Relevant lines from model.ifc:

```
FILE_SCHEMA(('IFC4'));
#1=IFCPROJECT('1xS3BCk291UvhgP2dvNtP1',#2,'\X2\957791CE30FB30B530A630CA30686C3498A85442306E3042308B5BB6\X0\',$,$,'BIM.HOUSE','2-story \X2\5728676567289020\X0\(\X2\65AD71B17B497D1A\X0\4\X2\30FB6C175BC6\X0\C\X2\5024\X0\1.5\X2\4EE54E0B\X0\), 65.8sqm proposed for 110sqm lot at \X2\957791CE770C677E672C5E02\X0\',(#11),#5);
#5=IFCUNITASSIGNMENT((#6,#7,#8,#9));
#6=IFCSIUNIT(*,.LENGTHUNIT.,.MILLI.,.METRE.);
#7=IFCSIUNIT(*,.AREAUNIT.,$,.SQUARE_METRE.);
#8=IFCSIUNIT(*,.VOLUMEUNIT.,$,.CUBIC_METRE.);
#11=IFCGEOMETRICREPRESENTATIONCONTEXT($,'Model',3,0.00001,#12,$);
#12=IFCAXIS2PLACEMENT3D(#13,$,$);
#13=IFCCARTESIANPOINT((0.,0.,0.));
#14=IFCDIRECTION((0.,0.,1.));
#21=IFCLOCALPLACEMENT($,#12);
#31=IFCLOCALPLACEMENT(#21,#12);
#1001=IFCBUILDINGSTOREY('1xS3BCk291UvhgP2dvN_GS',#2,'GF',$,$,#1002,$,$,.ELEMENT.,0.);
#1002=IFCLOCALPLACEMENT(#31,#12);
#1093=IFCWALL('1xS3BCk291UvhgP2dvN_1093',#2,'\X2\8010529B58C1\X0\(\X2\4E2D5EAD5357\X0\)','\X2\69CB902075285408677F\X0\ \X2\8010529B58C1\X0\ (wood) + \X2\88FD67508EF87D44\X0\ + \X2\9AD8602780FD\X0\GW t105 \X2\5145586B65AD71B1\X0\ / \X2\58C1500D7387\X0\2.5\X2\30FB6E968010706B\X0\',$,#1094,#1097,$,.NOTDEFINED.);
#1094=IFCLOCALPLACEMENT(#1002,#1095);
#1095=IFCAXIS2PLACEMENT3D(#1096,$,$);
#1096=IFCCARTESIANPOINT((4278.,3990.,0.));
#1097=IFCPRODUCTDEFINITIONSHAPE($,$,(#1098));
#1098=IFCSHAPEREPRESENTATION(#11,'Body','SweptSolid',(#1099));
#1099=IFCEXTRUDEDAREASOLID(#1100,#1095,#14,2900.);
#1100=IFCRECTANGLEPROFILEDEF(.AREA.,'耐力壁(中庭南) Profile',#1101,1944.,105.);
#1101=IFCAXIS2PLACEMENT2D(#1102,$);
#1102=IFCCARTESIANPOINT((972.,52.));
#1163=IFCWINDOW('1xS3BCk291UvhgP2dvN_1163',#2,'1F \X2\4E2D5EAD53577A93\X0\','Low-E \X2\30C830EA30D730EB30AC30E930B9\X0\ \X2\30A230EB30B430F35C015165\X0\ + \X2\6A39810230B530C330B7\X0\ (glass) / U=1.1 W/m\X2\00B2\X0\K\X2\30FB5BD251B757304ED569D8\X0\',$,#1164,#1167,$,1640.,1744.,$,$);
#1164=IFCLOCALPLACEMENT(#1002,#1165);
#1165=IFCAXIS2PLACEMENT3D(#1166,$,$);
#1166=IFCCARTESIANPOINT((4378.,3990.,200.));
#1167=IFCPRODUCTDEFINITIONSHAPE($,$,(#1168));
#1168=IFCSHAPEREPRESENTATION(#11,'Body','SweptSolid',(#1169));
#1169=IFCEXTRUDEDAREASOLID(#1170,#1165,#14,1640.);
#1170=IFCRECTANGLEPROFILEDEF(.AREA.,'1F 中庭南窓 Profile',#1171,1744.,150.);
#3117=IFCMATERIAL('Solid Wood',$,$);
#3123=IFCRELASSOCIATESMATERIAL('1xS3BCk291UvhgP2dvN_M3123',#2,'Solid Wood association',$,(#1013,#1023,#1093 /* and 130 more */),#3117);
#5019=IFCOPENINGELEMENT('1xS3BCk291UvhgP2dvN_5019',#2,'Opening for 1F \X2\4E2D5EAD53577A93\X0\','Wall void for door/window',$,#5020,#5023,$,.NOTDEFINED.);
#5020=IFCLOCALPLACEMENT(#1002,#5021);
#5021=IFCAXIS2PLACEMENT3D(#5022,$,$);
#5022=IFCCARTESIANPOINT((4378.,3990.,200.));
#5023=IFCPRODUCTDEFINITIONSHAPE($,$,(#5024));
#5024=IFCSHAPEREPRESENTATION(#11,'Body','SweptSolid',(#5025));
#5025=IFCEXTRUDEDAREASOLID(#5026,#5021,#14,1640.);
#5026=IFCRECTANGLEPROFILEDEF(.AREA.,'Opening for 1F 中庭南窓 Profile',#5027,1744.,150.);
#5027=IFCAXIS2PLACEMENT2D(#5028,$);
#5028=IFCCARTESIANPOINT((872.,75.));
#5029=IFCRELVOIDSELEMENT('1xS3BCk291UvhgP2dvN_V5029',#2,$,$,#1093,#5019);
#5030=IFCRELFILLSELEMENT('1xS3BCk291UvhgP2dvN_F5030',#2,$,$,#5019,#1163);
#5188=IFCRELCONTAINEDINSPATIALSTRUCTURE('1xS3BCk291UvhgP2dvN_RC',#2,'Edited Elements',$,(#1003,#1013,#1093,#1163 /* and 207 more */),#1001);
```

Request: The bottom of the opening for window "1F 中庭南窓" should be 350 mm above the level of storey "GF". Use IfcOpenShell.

```python
import numpy as np
import ifcopenshell
import ifcopenshell.api.geometry
import ifcopenshell.geom
import ifcopenshell.util.element
import ifcopenshell.util.placement
import ifcopenshell.util.shape
import ifcopenshell.util.unit

model = ifcopenshell.open("model.ifc")
unit_scale = ifcopenshell.util.unit.calculate_unit_scale(model)

window = model.by_guid("1xS3BCk291UvhgP2dvN_1163")
opening = window.FillsVoids[0].RelatingOpeningElement
storey = ifcopenshell.util.element.get_container(window, ifc_class="IfcBuildingStorey")
level = ifcopenshell.util.placement.get_local_placement(storey.ObjectPlacement)[2, 3]

# The opening's origin need not be at the sill, so measure its lowest point.
shape = ifcopenshell.geom.create_shape(ifcopenshell.geom.settings(), opening)
bottom = ifcopenshell.util.shape.get_shape_bottom_elevation(shape, shape.geometry) / unit_scale
dz = level + 0.35 / unit_scale - bottom

shift = np.array([0.0, 0.0, dz])
# The window is not placed relative to its opening, so move both.
for product in (opening, window):
    matrix = ifcopenshell.util.placement.get_local_placement(product.ObjectPlacement)
    matrix[:3, 3] += shift
    ifcopenshell.api.geometry.edit_object_placement(model, product=product, matrix=matrix, is_si=False)

print(f"moved by {dz * unit_scale:+.3f} m")

model.write("model_rev.ifc")
```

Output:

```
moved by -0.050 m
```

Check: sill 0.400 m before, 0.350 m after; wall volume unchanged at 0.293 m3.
